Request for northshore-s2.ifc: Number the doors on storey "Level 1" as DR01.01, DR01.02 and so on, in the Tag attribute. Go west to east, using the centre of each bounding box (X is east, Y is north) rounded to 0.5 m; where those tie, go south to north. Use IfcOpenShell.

First a look at what the model holds.

```python
import ifcopenshell
import ifcopenshell.util.element
import ifcopenshell.util.placement

model = ifcopenshell.open("northshore-s2.ifc")
print(model.schema)
storey = next(s for s in model.by_type("IfcBuildingStorey") if s.Name == "Level 1")
doors = [e for e in ifcopenshell.util.element.get_decomposition(storey) if e.is_a("IfcDoor")]
for e in sorted(doors, key=lambda e: e.id()):
    origin = ifcopenshell.util.placement.get_local_placement(e.ObjectPlacement)[:3, 3]
    print(e.id(), e.Tag, e.Name, origin.round(2) + 0.0, sep=" | ")
```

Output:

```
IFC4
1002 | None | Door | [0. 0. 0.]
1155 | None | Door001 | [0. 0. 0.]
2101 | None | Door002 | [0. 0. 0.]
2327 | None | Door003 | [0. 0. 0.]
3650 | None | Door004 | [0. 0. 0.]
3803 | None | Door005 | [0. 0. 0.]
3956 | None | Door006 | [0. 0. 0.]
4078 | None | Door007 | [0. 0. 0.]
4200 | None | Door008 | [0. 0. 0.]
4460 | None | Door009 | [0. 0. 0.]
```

```python
import ifcopenshell
import ifcopenshell.geom
import ifcopenshell.util.element
import ifcopenshell.util.shape

model = ifcopenshell.open("northshore-s2.ifc")
settings = ifcopenshell.geom.settings()
settings.set("use-world-coords", True)


def centre(element):
    shape = ifcopenshell.geom.create_shape(settings, element)
    return ifcopenshell.util.shape.get_bbox_centroid(shape.geometry)


storey = next(s for s in model.by_type("IfcBuildingStorey") if s.Name == "Level 1")
doors = [e for e in ifcopenshell.util.element.get_decomposition(storey) if e.is_a("IfcDoor")]

# Insertion points can sit at a corner or the storey origin, so sort by the geometry (in metres).
centres = {e: centre(e) for e in doors}
doors.sort(key=lambda e: (round(centres[e][0] / 0.5), centres[e][1]))

for i, e in enumerate(doors, start=1):
    number = f"DR01.{i:02d}"
    e.Tag = number
    print(e.id(), number)

model.write("northshore-s2-out.ifc")
```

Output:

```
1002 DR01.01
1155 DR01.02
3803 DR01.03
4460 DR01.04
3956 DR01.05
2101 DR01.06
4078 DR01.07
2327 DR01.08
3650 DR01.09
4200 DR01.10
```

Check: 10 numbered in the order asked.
